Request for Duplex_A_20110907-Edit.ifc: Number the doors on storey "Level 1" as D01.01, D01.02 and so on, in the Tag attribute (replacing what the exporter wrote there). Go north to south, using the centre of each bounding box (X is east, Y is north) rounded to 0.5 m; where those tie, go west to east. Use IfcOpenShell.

First a look at what the model holds.

```python
import ifcopenshell
import ifcopenshell.util.element
import ifcopenshell.util.placement

model = ifcopenshell.open("Duplex_A_20110907-Edit.ifc")
print(model.schema)
storey = next(s for s in model.by_type("IfcBuildingStorey") if s.Name == "Level 1")
doors = [e for e in ifcopenshell.util.element.get_decomposition(storey) if e.is_a("IfcDoor")]
for e in sorted(doors, key=lambda e: e.id()):
    origin = ifcopenshell.util.placement.get_local_placement(e.ObjectPlacement)[:3, 3]
    print(e.id(), e.Tag, e.Name, origin.round(2) + 0.0, sep=" | ")
```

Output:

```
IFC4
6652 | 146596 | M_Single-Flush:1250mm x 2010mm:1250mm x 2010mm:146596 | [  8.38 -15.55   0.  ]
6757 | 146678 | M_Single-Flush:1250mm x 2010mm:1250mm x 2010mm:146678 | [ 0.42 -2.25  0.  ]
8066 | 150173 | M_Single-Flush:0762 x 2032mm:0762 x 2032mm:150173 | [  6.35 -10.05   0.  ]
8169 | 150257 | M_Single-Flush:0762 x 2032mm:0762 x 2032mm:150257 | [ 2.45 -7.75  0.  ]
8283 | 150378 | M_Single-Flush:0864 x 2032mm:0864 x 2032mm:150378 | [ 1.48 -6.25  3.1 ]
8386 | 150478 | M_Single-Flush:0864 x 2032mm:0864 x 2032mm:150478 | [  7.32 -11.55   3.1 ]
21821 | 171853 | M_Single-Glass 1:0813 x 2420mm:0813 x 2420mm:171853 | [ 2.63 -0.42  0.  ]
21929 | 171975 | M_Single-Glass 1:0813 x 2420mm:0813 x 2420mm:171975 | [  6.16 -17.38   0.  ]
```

```python
import ifcopenshell
import ifcopenshell.geom
import ifcopenshell.util.element
import ifcopenshell.util.shape

model = ifcopenshell.open("Duplex_A_20110907-Edit.ifc")
settings = ifcopenshell.geom.settings()
settings.set("use-world-coords", True)


def centre(element):
    shape = ifcopenshell.geom.create_shape(settings, element)
    return ifcopenshell.util.shape.get_bbox_centroid(shape.geometry)


storey = next(s for s in model.by_type("IfcBuildingStorey") if s.Name == "Level 1")
doors = [e for e in ifcopenshell.util.element.get_decomposition(storey) if e.is_a("IfcDoor")]

# Insertion points can sit at a corner or the storey origin, so sort by the geometry (in metres).
centres = {e: centre(e) for e in doors}
doors.sort(key=lambda e: (-round(centres[e][1] / 0.5), centres[e][0]))

for i, e in enumerate(doors, start=1):
    number = f"D01.{i:02d}"
    e.Tag = number
    print(e.id(), number)

model.write("Duplex_A_20110907-Edit-out.ifc")
```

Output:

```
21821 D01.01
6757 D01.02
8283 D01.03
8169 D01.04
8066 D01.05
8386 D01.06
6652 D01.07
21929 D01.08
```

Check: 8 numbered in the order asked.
